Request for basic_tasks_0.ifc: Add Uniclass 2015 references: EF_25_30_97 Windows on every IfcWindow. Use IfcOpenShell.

First a look at what the model holds.

```python
import ifcopenshell

model = ifcopenshell.open("basic_tasks_0.ifc")
print(model.schema)
print("classifications:", [c.Name for c in model.by_type("IfcClassification")])
for ifc_class in ("IfcDoor", "IfcRoof", "IfcStair", "IfcWall", "IfcWindow"):
    print(ifc_class, len(model.by_type(ifc_class)))
```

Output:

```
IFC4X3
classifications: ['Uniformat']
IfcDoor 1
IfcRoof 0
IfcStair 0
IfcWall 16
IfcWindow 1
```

```python
import ifcopenshell
import ifcopenshell.api.classification

model = ifcopenshell.open("basic_tasks_0.ifc")

system = ifcopenshell.api.classification.add_classification(model, classification="Uniclass 2015")

codes = {
    "IfcWindow": ("EF_25_30_97", "Windows"),
}
for ifc_class, (code, name) in codes.items():
    products = model.by_type(ifc_class)
    ifcopenshell.api.classification.add_reference(
        model, products=products, classification=system, identification=code, name=name
    )
    print(code, len(products))

model.write("basic_tasks_0-out.ifc")
```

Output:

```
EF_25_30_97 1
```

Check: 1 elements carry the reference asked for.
